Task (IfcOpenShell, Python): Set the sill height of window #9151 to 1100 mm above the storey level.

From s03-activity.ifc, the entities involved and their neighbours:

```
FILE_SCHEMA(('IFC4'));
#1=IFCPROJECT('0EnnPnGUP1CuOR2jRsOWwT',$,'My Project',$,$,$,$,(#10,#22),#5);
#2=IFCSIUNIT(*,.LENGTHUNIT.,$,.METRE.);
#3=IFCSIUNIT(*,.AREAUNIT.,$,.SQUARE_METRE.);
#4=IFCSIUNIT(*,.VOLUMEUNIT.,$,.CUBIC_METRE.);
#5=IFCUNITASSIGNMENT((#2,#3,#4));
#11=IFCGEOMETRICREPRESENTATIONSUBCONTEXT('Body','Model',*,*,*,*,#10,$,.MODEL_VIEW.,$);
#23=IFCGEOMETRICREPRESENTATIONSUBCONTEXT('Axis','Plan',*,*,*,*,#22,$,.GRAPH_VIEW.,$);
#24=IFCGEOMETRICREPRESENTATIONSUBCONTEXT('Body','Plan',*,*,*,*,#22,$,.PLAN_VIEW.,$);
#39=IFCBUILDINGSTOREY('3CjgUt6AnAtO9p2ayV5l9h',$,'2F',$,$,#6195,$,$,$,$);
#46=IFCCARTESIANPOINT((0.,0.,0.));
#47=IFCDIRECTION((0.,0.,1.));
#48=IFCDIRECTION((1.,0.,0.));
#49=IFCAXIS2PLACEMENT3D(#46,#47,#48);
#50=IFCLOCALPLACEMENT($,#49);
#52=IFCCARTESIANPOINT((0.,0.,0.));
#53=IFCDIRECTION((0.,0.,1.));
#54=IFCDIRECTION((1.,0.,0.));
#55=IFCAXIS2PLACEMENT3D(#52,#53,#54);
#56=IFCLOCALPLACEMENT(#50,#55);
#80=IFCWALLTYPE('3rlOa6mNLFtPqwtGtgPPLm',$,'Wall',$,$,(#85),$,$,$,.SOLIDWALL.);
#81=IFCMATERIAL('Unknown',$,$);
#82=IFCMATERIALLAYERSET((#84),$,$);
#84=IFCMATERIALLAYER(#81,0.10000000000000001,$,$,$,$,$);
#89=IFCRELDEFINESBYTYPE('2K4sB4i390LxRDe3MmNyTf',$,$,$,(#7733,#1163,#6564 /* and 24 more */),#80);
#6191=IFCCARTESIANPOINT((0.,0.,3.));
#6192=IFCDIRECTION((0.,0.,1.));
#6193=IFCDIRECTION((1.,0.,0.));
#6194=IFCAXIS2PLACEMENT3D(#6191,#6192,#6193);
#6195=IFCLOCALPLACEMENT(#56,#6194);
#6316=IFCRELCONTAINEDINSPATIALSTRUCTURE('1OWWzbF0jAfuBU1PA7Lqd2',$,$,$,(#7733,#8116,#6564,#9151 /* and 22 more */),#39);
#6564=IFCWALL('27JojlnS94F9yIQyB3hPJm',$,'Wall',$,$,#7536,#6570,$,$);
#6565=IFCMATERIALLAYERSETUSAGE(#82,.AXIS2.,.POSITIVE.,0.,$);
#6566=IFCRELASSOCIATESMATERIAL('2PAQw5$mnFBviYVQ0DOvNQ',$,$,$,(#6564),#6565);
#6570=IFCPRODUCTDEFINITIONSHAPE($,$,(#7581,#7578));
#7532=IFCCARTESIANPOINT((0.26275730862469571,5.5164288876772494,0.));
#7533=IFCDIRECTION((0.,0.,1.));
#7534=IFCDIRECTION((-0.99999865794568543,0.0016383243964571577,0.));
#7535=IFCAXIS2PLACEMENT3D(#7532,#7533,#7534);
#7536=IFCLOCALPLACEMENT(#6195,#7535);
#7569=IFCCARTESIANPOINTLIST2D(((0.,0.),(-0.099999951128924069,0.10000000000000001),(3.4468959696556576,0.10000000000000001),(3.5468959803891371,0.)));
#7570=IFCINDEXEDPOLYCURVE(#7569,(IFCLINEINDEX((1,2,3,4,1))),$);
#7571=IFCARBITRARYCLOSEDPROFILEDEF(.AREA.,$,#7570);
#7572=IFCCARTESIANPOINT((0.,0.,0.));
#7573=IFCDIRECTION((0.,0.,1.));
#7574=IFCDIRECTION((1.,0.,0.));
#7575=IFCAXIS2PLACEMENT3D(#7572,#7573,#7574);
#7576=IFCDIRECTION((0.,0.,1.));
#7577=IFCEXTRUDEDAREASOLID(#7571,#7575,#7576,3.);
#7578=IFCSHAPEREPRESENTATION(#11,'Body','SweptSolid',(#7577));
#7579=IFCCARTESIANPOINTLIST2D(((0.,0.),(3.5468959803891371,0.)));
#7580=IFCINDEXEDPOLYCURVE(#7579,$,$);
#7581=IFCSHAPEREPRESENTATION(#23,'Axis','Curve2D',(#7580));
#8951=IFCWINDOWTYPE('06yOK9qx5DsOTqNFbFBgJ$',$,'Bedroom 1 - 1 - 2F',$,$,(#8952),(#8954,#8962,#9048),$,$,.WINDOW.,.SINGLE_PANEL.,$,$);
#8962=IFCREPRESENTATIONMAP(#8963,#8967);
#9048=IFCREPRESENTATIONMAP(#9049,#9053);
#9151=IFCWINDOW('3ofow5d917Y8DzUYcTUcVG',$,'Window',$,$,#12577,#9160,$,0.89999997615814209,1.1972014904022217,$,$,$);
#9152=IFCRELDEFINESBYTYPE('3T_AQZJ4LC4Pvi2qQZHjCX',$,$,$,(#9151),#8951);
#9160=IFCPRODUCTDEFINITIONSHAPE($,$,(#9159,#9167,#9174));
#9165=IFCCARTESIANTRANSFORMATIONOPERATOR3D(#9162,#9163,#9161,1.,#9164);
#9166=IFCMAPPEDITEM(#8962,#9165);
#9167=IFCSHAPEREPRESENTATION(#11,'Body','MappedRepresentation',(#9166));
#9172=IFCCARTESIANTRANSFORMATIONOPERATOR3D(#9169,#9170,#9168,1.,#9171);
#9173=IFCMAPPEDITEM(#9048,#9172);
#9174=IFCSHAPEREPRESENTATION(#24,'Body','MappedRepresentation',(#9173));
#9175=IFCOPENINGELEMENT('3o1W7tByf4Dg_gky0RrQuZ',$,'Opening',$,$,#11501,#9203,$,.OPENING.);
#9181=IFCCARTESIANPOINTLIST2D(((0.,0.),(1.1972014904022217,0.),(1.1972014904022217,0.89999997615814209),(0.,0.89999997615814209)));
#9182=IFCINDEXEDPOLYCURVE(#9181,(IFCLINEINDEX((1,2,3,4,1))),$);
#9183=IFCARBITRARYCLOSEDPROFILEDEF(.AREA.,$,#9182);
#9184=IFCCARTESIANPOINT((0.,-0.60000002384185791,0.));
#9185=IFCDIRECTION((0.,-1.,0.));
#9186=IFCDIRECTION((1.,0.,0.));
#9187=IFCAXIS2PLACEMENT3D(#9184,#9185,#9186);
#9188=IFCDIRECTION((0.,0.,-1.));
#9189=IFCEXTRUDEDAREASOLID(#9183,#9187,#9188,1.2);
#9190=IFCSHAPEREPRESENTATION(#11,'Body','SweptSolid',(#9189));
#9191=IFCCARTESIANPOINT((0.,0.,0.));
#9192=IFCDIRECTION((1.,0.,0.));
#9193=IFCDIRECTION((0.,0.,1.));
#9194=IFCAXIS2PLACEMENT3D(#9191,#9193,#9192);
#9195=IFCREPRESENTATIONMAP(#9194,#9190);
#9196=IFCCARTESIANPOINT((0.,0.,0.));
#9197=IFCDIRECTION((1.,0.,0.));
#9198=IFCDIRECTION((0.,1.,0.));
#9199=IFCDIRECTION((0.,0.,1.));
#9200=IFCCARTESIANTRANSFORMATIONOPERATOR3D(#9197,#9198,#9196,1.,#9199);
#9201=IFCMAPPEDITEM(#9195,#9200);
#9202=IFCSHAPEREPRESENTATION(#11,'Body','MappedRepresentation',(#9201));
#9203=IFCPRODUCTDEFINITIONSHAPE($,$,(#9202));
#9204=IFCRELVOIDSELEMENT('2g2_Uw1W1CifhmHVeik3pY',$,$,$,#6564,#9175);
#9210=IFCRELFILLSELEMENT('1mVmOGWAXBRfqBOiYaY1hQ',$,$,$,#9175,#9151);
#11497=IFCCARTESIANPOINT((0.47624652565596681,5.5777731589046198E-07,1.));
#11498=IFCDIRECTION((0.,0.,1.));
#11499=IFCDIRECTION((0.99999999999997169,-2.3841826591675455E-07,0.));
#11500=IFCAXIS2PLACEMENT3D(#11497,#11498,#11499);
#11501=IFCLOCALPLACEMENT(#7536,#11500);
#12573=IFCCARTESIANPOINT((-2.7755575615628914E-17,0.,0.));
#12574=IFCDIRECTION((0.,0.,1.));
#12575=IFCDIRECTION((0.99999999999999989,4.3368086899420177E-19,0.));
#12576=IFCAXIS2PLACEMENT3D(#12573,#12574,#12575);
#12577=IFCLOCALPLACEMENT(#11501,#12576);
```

```python
import numpy as np
import ifcopenshell
import ifcopenshell.api.geometry
import ifcopenshell.geom
import ifcopenshell.util.element
import ifcopenshell.util.placement
import ifcopenshell.util.shape
import ifcopenshell.util.unit

model = ifcopenshell.open("s03-activity.ifc")
unit_scale = ifcopenshell.util.unit.calculate_unit_scale(model)

window = model.by_id(9151)
opening = window.FillsVoids[0].RelatingOpeningElement
storey = ifcopenshell.util.element.get_container(window, ifc_class="IfcBuildingStorey")
level = ifcopenshell.util.placement.get_local_placement(storey.ObjectPlacement)[2, 3]

# The opening's origin need not be at the sill, so measure its lowest point.
shape = ifcopenshell.geom.create_shape(ifcopenshell.geom.settings(), opening)
bottom = ifcopenshell.util.shape.get_shape_bottom_elevation(shape, shape.geometry) / unit_scale
dz = level + 1.1 - bottom

shift = np.array([0.0, 0.0, dz])
# The window is placed relative to its opening, so it follows when the opening moves.
matrix = ifcopenshell.util.placement.get_local_placement(opening.ObjectPlacement)
matrix[:3, 3] += shift
ifcopenshell.api.geometry.edit_object_placement(
    model, product=opening, matrix=matrix, is_si=False, should_transform_children=True
)

print(f"moved by {dz * unit_scale:+.3f} m")

model.write("s03-activity_edited.ifc")
```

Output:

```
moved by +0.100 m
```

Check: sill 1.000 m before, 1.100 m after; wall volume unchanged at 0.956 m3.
